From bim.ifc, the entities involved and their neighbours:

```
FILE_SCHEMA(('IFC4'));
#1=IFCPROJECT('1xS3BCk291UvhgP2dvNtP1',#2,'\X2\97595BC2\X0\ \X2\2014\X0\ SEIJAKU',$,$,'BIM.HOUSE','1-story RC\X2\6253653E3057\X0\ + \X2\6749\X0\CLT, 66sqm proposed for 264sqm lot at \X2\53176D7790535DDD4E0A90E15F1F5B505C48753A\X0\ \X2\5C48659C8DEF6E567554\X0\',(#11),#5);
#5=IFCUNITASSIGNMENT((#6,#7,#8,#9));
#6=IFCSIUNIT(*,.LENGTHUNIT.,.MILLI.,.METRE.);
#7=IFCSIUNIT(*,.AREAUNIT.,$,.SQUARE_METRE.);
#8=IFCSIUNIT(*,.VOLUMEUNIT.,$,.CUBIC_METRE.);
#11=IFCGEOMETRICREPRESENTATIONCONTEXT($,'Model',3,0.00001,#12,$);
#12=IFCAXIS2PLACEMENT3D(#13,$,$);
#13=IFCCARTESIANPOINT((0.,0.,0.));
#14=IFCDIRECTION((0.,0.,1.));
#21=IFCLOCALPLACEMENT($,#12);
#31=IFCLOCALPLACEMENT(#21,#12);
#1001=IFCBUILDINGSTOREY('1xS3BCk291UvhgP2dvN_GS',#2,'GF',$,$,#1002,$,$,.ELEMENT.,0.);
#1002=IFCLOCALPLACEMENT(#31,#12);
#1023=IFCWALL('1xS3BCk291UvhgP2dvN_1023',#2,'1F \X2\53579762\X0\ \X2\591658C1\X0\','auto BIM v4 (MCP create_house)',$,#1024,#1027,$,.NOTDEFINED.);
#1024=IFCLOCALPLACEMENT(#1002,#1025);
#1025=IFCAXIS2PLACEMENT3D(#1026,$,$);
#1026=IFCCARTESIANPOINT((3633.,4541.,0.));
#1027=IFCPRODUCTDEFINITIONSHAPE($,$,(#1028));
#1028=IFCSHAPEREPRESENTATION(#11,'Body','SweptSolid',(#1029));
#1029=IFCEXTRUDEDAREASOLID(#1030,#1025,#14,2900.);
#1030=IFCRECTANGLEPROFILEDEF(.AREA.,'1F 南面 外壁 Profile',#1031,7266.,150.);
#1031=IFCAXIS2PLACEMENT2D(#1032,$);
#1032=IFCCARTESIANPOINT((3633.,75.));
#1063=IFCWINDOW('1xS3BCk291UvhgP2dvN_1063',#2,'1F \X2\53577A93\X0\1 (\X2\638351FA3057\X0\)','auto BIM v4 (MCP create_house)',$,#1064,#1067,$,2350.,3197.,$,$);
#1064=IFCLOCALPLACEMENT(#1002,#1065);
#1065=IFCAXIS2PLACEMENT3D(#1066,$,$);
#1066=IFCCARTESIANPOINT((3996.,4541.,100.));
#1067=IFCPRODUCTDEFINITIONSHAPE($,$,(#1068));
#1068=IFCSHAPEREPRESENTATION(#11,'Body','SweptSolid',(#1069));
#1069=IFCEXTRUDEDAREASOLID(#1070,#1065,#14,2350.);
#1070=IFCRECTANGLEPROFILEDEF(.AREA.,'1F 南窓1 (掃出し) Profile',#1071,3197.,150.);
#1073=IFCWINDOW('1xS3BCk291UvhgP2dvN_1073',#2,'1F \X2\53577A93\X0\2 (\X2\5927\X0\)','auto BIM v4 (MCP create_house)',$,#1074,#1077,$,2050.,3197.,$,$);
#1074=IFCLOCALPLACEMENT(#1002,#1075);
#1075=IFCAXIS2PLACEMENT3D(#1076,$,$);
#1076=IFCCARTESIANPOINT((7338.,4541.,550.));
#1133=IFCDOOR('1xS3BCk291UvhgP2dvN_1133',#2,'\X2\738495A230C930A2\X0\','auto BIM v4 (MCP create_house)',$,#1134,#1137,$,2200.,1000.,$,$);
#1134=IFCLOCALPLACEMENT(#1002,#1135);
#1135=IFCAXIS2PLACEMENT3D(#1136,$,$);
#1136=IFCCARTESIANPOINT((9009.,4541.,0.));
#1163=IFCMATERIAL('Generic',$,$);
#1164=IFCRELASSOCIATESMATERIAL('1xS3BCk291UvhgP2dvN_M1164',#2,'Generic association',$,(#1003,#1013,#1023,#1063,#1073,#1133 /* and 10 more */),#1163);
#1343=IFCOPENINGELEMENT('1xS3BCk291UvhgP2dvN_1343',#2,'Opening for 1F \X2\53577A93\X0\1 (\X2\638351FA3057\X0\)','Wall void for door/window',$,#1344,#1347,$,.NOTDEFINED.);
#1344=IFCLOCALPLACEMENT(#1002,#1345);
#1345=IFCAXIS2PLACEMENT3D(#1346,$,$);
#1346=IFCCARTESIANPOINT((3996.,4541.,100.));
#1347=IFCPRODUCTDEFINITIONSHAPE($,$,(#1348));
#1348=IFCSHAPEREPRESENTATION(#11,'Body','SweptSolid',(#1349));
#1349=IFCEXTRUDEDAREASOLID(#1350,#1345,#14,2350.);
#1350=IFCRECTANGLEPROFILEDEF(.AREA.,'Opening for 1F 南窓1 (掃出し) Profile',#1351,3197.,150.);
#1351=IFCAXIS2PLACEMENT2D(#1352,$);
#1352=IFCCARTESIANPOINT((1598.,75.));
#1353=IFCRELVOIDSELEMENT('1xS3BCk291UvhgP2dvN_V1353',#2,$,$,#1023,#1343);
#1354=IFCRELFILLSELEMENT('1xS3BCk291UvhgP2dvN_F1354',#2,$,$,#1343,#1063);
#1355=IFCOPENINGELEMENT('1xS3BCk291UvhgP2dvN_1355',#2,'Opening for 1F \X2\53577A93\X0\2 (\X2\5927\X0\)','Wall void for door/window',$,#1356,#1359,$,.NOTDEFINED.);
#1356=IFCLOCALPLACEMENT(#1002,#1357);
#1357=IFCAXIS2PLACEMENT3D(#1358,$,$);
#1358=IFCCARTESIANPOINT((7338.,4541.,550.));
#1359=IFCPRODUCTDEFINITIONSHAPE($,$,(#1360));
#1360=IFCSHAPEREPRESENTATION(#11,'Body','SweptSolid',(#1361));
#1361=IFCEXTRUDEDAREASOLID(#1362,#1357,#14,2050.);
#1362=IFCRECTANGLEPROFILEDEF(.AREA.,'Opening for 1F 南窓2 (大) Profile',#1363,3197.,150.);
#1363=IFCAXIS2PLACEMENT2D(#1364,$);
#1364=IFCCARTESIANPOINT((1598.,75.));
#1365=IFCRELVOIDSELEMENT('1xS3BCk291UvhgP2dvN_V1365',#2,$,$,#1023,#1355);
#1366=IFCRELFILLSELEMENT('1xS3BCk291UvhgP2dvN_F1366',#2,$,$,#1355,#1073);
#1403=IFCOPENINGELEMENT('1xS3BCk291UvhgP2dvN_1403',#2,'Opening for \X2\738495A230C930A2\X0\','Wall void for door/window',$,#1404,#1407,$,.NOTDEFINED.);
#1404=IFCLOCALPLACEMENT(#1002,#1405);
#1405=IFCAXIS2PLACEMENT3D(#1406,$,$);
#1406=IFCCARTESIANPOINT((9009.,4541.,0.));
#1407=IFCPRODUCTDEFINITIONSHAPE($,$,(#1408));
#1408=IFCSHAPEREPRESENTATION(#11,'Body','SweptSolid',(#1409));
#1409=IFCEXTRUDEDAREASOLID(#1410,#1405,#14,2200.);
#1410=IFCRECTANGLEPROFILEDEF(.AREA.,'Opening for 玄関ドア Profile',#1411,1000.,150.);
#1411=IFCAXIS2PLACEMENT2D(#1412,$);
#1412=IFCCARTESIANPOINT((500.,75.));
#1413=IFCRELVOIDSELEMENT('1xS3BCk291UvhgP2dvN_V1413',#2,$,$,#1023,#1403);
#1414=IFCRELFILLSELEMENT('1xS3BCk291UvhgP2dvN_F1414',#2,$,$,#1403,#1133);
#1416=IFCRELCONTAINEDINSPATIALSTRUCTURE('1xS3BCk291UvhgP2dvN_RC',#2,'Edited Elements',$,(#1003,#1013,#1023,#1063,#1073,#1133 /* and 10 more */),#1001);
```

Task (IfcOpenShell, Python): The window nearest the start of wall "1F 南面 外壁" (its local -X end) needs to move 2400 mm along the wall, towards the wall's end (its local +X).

```python
import ifcopenshell
import ifcopenshell.api.geometry
import ifcopenshell.util.placement
import ifcopenshell.util.unit

model = ifcopenshell.open("bim.ifc")
unit_scale = ifcopenshell.util.unit.calculate_unit_scale(model)

window = model.by_guid("1xS3BCk291UvhgP2dvN_1063")
opening = window.FillsVoids[0].RelatingOpeningElement
wall = opening.VoidsElements[0].RelatingBuildingElement

wall_matrix = ifcopenshell.util.placement.get_local_placement(wall.ObjectPlacement)
shift = wall_matrix[:3, 0] * 2.4 / unit_scale
before = ifcopenshell.util.placement.get_local_placement(window.ObjectPlacement)[:3, 3].copy()

# The window is not placed relative to its opening, so move both.
for product in (opening, window):
    matrix = ifcopenshell.util.placement.get_local_placement(product.ObjectPlacement)
    matrix[:3, 3] += shift
    ifcopenshell.api.geometry.edit_object_placement(model, product=product, matrix=matrix, is_si=False)

after = ifcopenshell.util.placement.get_local_placement(window.ObjectPlacement)[:3, 3]
print("window moved by", (after - before).round(3) + 0.0)

model.write("bim_v2.ifc")
```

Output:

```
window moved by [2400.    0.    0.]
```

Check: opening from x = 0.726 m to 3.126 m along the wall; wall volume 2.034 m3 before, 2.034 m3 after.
